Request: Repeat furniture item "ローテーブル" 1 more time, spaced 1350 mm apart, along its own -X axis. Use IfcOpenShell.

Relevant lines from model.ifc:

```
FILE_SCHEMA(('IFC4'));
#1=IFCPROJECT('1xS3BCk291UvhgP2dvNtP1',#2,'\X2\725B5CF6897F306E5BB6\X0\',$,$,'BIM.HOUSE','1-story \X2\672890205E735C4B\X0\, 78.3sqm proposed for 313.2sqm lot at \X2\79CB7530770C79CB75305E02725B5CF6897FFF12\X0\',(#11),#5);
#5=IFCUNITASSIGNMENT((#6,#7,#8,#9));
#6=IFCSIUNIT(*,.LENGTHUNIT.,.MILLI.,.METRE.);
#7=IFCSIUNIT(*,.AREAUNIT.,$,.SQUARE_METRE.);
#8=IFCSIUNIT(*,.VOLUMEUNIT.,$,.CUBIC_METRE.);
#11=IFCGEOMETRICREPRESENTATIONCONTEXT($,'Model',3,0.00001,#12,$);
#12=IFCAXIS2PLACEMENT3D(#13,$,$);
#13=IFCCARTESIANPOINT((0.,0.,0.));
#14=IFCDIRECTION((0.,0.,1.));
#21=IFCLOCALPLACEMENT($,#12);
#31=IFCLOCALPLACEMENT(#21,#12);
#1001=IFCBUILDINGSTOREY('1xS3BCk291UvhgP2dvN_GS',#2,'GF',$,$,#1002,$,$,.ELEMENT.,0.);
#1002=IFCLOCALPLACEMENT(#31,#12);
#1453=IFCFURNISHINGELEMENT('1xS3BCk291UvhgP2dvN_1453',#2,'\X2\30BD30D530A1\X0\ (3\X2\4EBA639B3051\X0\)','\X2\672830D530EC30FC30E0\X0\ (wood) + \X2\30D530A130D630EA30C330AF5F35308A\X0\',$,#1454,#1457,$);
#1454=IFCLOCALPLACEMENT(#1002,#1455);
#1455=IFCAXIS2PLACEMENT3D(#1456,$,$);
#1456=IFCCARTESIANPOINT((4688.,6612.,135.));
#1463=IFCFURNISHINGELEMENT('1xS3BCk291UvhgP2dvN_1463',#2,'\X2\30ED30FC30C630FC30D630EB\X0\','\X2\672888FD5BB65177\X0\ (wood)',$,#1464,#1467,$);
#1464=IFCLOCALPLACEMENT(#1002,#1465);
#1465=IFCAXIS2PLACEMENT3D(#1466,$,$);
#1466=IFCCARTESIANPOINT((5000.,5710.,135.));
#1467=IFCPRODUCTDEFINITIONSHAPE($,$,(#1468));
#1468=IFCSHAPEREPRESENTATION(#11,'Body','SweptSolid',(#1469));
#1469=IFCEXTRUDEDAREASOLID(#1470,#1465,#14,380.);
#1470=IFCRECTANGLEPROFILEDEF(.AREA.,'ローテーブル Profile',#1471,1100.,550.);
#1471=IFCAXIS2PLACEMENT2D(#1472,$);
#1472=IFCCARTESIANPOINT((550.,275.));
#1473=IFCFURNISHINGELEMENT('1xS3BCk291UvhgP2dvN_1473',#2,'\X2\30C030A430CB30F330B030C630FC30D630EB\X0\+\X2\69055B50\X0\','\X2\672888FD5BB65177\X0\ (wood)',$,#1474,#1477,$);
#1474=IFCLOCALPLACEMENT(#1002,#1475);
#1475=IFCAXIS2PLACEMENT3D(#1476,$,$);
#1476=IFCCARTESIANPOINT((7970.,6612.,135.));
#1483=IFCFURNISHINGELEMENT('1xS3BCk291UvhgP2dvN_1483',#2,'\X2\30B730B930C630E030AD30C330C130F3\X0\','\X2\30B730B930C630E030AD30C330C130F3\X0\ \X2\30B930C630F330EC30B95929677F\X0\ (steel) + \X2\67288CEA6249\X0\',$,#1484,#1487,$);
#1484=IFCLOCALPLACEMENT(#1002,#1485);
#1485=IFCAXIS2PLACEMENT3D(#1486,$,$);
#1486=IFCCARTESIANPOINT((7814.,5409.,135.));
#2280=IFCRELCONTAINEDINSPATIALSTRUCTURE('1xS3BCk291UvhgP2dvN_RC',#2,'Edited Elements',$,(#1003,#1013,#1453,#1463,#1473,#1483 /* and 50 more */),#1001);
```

```python
import ifcopenshell
import ifcopenshell.api.geometry
import ifcopenshell.api.root
import ifcopenshell.util.element
import ifcopenshell.util.placement

model = ifcopenshell.open("model.ifc")


def reuse_history(source, copy):
    """copy_class also copies each property set's owner history, people and application; keep the originals."""
    for rel in copy.IsDefinedBy:
        if rel.is_a("IfcRelDefinesByProperties") and (history := rel.RelatingPropertyDefinition.OwnerHistory):
            rel.RelatingPropertyDefinition.OwnerHistory = source.OwnerHistory
            ifcopenshell.util.element.remove_deep2(model, history)


source = model.by_id(1463)
base = ifcopenshell.util.placement.get_local_placement(source.ObjectPlacement)
step = -base[:3, 0] * 1350.0

for i in range(1, 2):
    copy = ifcopenshell.api.root.copy_class(model, product=source)
    copy.Representation = ifcopenshell.util.element.copy_deep(
        model, source.Representation, exclude=["IfcGeometricRepresentationContext", "IfcRepresentationMap"]
    )
    reuse_history(source, copy)
    matrix = base.copy()
    matrix[:3, 3] += i * step
    print("added at", matrix[:3, 3].round(3) + 0.0)
    ifcopenshell.api.geometry.edit_object_placement(model, product=copy, matrix=matrix, is_si=False)

model.write("model_v2.ifc")
```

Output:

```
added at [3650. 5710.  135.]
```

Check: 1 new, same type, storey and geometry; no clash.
